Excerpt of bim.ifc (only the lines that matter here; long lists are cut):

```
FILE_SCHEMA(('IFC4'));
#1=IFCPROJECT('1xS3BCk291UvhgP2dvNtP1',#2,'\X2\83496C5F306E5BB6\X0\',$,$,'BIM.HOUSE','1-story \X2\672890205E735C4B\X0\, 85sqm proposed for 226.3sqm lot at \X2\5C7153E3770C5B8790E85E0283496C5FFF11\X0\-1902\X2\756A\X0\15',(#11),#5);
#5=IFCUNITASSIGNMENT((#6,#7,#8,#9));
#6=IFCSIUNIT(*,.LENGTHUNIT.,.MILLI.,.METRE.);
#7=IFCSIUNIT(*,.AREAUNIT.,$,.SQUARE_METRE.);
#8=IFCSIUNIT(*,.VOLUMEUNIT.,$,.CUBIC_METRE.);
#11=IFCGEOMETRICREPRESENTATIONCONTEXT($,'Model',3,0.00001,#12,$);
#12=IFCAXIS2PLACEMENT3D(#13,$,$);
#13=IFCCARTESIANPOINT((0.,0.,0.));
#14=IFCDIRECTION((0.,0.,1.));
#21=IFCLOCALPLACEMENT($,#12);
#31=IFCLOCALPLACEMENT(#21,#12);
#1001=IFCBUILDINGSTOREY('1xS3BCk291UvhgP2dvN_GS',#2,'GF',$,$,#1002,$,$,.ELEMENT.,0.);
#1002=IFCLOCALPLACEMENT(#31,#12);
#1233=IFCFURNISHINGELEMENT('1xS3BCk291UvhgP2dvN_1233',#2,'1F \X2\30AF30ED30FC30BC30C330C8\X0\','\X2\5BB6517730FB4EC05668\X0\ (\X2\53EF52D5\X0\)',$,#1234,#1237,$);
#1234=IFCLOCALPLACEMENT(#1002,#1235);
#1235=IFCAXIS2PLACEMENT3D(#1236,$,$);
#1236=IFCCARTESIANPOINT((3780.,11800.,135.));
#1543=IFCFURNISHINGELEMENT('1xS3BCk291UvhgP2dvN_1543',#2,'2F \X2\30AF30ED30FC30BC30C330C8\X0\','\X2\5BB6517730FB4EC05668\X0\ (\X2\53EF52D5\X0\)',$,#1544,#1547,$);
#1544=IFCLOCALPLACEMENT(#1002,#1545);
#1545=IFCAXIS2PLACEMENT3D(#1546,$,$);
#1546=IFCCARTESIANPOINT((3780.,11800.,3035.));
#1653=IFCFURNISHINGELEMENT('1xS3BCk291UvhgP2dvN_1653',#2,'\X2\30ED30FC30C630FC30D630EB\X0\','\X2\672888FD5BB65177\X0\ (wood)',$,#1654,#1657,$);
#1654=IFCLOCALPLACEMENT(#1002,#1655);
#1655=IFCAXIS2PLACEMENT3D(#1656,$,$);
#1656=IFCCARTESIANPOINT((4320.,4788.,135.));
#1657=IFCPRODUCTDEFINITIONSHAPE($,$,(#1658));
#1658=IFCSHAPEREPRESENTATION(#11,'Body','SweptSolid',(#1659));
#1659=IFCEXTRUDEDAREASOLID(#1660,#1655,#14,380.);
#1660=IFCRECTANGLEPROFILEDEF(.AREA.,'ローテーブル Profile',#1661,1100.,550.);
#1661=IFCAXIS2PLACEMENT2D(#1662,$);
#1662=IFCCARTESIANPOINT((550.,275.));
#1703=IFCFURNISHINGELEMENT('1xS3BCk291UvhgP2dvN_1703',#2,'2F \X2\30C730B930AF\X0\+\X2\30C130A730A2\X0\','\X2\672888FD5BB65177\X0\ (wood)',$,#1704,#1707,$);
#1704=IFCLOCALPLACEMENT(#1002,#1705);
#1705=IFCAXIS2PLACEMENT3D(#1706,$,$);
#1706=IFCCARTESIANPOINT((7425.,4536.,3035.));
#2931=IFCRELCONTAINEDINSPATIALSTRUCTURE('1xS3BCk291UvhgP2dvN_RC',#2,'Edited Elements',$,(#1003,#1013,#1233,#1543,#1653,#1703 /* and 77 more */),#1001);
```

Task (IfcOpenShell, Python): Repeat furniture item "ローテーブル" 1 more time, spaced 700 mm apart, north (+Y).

```python
import numpy as np
import ifcopenshell
import ifcopenshell.api.geometry
import ifcopenshell.api.root
import ifcopenshell.util.element
import ifcopenshell.util.placement
import ifcopenshell.util.unit

model = ifcopenshell.open("bim.ifc")
unit_scale = ifcopenshell.util.unit.calculate_unit_scale(model)


def reuse_history(source, copy):
    """copy_class also copies each property set's owner history, people and application; keep the originals."""
    for rel in copy.IsDefinedBy:
        if rel.is_a("IfcRelDefinesByProperties") and (history := rel.RelatingPropertyDefinition.OwnerHistory):
            rel.RelatingPropertyDefinition.OwnerHistory = source.OwnerHistory
            ifcopenshell.util.element.remove_deep2(model, history)


source = model.by_id(1653)
base = ifcopenshell.util.placement.get_local_placement(source.ObjectPlacement)
step = np.array([0.0, 1.0, 0.0]) * 0.7 / unit_scale

for i in range(1, 2):
    copy = ifcopenshell.api.root.copy_class(model, product=source)
    copy.Representation = ifcopenshell.util.element.copy_deep(
        model, source.Representation, exclude=["IfcGeometricRepresentationContext", "IfcRepresentationMap"]
    )
    reuse_history(source, copy)
    matrix = base.copy()
    matrix[:3, 3] += i * step
    print("added at", matrix[:3, 3].round(3) + 0.0)
    ifcopenshell.api.geometry.edit_object_placement(model, product=copy, matrix=matrix, is_si=False)

model.write("bim_edited.ifc")
```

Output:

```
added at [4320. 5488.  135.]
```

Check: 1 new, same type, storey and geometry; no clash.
